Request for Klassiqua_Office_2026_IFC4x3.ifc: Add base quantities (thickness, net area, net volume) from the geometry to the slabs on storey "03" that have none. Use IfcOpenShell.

First a look at what the model holds.

```python
import ifcopenshell
import ifcopenshell.util.element
import ifcopenshell.util.unit

model = ifcopenshell.open("Klassiqua_Office_2026_IFC4x3.ifc")
print(model.schema)
for unit_type in ("LENGTHUNIT", "AREAUNIT", "VOLUMEUNIT"):
    print(unit_type, ifcopenshell.util.unit.calculate_unit_scale(model, unit_type))
storey = next(s for s in model.by_type("IfcBuildingStorey") if s.Name == "03")
slabs = [e for e in ifcopenshell.util.element.get_decomposition(storey) if e.is_a("IfcSlab")]
for e in sorted(slabs, key=lambda e: e.id()):
    print(e.id(), e.is_a(), e.Name, list(ifcopenshell.util.element.get_psets(e, qtos_only=True)), sep=" | ")
```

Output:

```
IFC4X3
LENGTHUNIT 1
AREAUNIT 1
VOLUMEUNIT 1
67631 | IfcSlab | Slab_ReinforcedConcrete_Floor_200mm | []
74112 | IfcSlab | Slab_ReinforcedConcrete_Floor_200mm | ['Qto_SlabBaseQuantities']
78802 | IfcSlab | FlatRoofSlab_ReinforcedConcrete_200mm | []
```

```python
import ifcopenshell
import ifcopenshell.api.pset
import ifcopenshell.geom
import ifcopenshell.util.element
import ifcopenshell.util.shape
import ifcopenshell.util.unit

model = ifcopenshell.open("Klassiqua_Office_2026_IFC4x3.ifc")
unit_scale = ifcopenshell.util.unit.calculate_unit_scale(model)
area_scale = ifcopenshell.util.unit.calculate_unit_scale(model, "AREAUNIT")
volume_scale = ifcopenshell.util.unit.calculate_unit_scale(model, "VOLUMEUNIT")
settings = ifcopenshell.geom.settings()

storey = next(s for s in model.by_type("IfcBuildingStorey") if s.Name == "03")
slabs = [e for e in ifcopenshell.util.element.get_decomposition(storey) if e.is_a("IfcSlab")]

for e in sorted(slabs, key=lambda e: e.id()):
    if ifcopenshell.util.element.get_psets(e, qtos_only=True, should_inherit=False):
        continue
    # Geometry comes back in metres, in the element's own axes.
    shape = ifcopenshell.geom.create_shape(settings, e)
    values = {
        "Width": ifcopenshell.util.shape.get_z(shape.geometry) / unit_scale,
        "NetArea": ifcopenshell.util.shape.get_footprint_area(shape.geometry) / area_scale,
        "NetVolume": ifcopenshell.util.shape.get_volume(shape.geometry) / volume_scale,
    }
    qto = ifcopenshell.api.pset.add_qto(model, product=e, name="Qto_SlabBaseQuantities")
    ifcopenshell.api.pset.edit_qto(model, qto=qto, properties=values)
    print(e.id(), {k: round(v, 3) for k, v in values.items()})

model.write("Klassiqua_Office_2026_IFC4x3-out.ifc")
```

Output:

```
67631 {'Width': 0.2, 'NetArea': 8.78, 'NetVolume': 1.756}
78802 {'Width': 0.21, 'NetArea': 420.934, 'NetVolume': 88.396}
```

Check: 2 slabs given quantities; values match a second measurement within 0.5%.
